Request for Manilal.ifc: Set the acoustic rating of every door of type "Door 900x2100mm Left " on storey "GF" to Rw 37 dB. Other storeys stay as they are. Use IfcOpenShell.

First a look at what the model holds.

```python
import ifcopenshell
import ifcopenshell.util.element

model = ifcopenshell.open("Manilal.ifc")
print(model.schema)
storey = next(s for s in model.by_type("IfcBuildingStorey") if s.Name == "GF")
doors = [e for e in ifcopenshell.util.element.get_decomposition(storey) if e.is_a("IfcDoor")]
seen = {}
for e in doors:
    element_type = ifcopenshell.util.element.get_type(e)
    key = (element_type.Name if element_type != e and element_type else None, ifcopenshell.util.element.get_pset(e, "Pset_DoorCommon", "AcousticRating"))
    seen[key] = seen.get(key, 0) + 1
for (name, value), count in sorted(seen.items(), key=str):
    print(count, "x", name, "|", value)
```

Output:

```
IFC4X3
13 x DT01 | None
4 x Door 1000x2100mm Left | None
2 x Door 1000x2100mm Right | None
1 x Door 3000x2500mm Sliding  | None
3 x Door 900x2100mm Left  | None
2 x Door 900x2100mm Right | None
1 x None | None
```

```python
import ifcopenshell
import ifcopenshell.api.pset
import ifcopenshell.util.element

model = ifcopenshell.open("Manilal.ifc")

storey = next(s for s in model.by_type("IfcBuildingStorey") if s.Name == "GF")
doors = [e for e in ifcopenshell.util.element.get_decomposition(storey) if e.is_a("IfcDoor")]

count = 0
for e in doors:
    element_type = ifcopenshell.util.element.get_type(e)
    if element_type in (None, e) or element_type.Name != "Door 900x2100mm Left ":
        continue
    # add_pset returns the element's existing set when there is one.
    pset = ifcopenshell.api.pset.add_pset(model, product=e, name="Pset_DoorCommon")
    ifcopenshell.api.pset.edit_pset(model, pset=pset, properties={"AcousticRating": "Rw 37 dB"})
    count += 1

print(count, "doors updated")

model.write("Manilal_updated.ifc")
```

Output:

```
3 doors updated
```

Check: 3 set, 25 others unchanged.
